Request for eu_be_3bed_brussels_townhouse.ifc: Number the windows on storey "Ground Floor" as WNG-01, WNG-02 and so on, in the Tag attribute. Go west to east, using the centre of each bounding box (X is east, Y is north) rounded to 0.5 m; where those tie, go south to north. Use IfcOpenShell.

First a look at what the model holds.

```python
import ifcopenshell
import ifcopenshell.util.element
import ifcopenshell.util.placement

model = ifcopenshell.open("eu_be_3bed_brussels_townhouse.ifc")
print(model.schema)
storey = next(s for s in model.by_type("IfcBuildingStorey") if s.Name == "Ground Floor")
windows = [e for e in ifcopenshell.util.element.get_decomposition(storey) if e.is_a("IfcWindow")]
for e in sorted(windows, key=lambda e: e.id()):
    origin = ifcopenshell.util.placement.get_local_placement(e.ObjectPlacement)[:3, 3]
    print(e.id(), e.Tag, e.Name, origin.round(2) + 0.0, sep=" | ")
```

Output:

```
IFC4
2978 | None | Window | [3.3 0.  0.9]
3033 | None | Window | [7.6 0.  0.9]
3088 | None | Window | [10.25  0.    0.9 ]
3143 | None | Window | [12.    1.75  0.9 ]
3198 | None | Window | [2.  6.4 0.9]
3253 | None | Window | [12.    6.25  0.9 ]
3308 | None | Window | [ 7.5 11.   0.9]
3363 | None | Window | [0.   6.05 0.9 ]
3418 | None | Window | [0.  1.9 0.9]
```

```python
import ifcopenshell
import ifcopenshell.geom
import ifcopenshell.util.element
import ifcopenshell.util.shape

model = ifcopenshell.open("eu_be_3bed_brussels_townhouse.ifc")
settings = ifcopenshell.geom.settings()
settings.set("use-world-coords", True)


def centre(element):
    shape = ifcopenshell.geom.create_shape(settings, element)
    return ifcopenshell.util.shape.get_bbox_centroid(shape.geometry)


storey = next(s for s in model.by_type("IfcBuildingStorey") if s.Name == "Ground Floor")
windows = [e for e in ifcopenshell.util.element.get_decomposition(storey) if e.is_a("IfcWindow")]

# Insertion points can sit at a corner or the storey origin, so sort by the geometry (in metres).
centres = {e: centre(e) for e in windows}
windows.sort(key=lambda e: (round(centres[e][0] / 0.5), centres[e][1]))

for i, e in enumerate(windows, start=1):
    number = f"WNG-{i:02d}"
    e.Tag = number
    print(e.id(), number)

model.write("eu_be_3bed_brussels_townhouse_edited.ifc")
```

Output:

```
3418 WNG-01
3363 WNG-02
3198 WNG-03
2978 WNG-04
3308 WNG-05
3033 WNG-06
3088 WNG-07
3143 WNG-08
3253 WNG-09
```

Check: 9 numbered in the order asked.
